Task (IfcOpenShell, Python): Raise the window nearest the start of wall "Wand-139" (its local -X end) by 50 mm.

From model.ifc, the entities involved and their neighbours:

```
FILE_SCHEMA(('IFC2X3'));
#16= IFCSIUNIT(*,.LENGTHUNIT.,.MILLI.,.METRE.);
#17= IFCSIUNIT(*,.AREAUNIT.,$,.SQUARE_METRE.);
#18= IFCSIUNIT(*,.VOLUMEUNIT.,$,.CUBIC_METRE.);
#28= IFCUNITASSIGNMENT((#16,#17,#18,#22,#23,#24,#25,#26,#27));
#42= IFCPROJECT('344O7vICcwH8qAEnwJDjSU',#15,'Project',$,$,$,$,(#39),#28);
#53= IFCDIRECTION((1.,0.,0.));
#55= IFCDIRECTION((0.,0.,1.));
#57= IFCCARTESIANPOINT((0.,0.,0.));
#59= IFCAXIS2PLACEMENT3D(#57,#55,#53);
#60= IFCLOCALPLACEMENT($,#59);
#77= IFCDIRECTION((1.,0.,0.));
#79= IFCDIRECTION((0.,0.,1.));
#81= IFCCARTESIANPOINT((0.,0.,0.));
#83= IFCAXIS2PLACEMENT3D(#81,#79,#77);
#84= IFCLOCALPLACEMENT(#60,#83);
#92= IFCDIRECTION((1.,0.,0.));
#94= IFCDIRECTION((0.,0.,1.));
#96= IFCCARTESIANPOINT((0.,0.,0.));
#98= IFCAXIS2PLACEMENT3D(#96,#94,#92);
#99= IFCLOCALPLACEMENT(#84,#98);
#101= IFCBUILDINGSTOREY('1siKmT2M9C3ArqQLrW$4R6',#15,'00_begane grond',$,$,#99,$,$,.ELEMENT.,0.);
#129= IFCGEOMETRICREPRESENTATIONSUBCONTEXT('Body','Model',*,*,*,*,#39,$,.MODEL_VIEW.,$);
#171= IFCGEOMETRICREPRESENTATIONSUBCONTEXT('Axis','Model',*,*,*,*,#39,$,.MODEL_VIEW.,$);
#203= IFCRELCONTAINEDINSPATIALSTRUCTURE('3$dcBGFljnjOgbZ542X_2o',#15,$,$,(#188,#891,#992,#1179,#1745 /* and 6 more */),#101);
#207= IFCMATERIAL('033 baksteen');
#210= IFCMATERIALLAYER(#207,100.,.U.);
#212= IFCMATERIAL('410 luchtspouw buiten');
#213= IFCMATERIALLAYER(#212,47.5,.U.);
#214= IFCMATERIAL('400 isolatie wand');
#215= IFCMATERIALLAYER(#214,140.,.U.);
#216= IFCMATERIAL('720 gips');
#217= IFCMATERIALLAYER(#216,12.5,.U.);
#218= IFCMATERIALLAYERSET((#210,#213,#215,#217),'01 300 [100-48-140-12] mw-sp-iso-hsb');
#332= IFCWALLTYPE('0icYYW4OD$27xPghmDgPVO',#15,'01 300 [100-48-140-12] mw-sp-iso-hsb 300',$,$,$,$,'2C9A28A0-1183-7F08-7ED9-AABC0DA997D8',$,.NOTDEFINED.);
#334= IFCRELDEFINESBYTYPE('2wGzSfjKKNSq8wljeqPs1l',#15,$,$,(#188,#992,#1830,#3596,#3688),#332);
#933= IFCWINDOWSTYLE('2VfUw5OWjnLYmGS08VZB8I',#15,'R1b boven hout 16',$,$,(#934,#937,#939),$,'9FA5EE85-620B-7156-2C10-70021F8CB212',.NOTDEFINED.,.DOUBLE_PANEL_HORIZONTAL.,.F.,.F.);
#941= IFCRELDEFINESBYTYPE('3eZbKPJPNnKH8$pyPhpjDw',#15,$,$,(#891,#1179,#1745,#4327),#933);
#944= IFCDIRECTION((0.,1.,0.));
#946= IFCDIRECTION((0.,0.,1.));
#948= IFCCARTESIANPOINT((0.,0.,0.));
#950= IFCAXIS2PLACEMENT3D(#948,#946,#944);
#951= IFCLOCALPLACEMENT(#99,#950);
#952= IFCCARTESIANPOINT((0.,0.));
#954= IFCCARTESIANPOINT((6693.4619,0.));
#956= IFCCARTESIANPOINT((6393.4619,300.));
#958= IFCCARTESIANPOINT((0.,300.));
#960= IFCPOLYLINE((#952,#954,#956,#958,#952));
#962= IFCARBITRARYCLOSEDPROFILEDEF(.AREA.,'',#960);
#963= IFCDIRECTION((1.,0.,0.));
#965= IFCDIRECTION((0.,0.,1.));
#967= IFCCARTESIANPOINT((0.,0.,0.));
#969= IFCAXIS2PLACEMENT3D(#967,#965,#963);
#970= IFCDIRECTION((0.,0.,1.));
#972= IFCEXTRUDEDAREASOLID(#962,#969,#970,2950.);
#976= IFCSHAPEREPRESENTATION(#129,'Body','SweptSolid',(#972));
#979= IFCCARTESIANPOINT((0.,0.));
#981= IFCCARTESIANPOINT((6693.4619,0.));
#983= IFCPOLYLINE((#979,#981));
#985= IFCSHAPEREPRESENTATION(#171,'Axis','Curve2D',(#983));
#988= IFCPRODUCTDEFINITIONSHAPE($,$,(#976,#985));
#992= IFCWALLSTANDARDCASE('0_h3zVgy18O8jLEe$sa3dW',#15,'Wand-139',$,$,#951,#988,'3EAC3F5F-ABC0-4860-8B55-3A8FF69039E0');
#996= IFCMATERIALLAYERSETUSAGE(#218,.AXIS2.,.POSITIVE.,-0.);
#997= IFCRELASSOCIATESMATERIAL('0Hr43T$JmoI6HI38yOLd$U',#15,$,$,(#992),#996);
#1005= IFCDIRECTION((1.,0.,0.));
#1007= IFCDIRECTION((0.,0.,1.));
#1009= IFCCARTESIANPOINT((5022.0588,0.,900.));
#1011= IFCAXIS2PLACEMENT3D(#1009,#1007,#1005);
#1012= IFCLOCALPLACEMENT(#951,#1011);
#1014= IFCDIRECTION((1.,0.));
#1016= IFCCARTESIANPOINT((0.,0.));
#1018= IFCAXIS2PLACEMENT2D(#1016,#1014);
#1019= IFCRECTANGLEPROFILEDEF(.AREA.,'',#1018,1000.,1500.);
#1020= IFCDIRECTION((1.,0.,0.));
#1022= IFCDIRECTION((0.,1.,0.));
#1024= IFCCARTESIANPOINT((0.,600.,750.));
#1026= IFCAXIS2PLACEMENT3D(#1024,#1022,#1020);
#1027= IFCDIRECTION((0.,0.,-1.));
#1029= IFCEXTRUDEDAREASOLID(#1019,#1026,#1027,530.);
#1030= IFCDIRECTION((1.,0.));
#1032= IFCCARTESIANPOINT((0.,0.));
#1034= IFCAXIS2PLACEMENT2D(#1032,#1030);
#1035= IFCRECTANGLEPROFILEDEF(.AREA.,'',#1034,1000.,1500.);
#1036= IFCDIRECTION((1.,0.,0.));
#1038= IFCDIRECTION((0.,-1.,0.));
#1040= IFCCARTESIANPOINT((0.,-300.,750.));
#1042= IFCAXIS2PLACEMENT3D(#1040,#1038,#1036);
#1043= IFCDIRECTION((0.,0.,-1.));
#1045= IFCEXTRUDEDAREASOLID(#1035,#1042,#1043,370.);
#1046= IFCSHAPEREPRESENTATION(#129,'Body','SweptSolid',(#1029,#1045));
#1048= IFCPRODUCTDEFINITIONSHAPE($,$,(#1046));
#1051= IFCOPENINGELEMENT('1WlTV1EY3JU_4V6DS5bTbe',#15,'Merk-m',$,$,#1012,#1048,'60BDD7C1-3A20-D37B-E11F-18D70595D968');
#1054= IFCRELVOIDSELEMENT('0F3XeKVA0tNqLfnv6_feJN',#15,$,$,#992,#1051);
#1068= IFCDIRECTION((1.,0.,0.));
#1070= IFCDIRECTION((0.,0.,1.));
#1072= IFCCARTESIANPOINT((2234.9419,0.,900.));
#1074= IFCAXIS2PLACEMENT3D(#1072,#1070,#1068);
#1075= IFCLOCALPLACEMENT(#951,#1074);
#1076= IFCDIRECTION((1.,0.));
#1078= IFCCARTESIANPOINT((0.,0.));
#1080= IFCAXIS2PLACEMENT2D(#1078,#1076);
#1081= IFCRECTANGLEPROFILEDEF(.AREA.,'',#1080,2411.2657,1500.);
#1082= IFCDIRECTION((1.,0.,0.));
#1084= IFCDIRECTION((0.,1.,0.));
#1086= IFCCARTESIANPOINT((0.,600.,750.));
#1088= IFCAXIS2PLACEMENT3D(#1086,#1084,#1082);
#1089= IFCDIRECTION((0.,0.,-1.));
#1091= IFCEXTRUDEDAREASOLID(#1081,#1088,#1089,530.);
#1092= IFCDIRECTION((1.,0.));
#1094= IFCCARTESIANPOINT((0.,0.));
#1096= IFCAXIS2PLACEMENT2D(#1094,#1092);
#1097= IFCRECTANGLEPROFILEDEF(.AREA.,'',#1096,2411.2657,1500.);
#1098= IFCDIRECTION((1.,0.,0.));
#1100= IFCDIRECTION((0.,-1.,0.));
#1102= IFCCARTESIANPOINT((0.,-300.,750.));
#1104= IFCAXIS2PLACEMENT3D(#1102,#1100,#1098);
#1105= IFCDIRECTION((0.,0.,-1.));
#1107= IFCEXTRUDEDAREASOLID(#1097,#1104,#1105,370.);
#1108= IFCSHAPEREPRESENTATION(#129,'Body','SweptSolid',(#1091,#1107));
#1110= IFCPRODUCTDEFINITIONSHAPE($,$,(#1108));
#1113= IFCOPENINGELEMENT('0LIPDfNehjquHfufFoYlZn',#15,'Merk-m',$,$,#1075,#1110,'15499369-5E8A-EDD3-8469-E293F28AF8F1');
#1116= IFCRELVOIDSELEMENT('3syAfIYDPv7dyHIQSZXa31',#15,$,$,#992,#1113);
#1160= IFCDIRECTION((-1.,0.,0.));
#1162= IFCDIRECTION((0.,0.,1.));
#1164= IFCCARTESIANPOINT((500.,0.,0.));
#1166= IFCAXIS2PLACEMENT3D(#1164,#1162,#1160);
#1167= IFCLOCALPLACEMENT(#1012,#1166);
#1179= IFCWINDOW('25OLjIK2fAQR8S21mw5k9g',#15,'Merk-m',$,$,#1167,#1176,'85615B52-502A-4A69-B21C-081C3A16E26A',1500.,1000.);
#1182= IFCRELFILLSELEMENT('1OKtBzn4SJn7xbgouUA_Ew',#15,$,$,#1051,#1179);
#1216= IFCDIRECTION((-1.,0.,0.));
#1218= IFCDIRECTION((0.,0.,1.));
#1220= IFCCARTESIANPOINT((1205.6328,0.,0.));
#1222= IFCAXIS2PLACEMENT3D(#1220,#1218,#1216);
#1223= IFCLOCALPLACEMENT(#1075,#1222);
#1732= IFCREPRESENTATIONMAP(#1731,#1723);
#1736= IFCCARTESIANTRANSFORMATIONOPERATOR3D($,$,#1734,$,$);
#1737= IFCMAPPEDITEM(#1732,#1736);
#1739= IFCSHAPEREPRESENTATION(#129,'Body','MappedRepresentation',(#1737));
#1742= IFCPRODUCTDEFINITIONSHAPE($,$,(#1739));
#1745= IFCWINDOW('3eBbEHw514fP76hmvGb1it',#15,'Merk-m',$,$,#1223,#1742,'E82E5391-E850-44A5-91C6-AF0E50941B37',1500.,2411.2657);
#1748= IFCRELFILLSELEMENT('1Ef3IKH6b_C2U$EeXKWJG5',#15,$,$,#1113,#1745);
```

```python
import numpy as np
import ifcopenshell
import ifcopenshell.api.geometry
import ifcopenshell.util.placement
import ifcopenshell.util.unit

model = ifcopenshell.open("model.ifc")
unit_scale = ifcopenshell.util.unit.calculate_unit_scale(model)

window = model.by_guid("3eBbEHw514fP76hmvGb1it")
opening = window.FillsVoids[0].RelatingOpeningElement
dz = 0.05 / unit_scale

shift = np.array([0.0, 0.0, dz])
# The window is placed relative to its opening, so it follows when the opening moves.
matrix = ifcopenshell.util.placement.get_local_placement(opening.ObjectPlacement)
matrix[:3, 3] += shift
ifcopenshell.api.geometry.edit_object_placement(
    model, product=opening, matrix=matrix, is_si=False, should_transform_children=True
)

print(f"moved by {dz * unit_scale:+.3f} m")

model.write("model_v2.ifc")
```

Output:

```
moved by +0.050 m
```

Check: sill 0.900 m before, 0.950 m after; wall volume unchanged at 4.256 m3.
